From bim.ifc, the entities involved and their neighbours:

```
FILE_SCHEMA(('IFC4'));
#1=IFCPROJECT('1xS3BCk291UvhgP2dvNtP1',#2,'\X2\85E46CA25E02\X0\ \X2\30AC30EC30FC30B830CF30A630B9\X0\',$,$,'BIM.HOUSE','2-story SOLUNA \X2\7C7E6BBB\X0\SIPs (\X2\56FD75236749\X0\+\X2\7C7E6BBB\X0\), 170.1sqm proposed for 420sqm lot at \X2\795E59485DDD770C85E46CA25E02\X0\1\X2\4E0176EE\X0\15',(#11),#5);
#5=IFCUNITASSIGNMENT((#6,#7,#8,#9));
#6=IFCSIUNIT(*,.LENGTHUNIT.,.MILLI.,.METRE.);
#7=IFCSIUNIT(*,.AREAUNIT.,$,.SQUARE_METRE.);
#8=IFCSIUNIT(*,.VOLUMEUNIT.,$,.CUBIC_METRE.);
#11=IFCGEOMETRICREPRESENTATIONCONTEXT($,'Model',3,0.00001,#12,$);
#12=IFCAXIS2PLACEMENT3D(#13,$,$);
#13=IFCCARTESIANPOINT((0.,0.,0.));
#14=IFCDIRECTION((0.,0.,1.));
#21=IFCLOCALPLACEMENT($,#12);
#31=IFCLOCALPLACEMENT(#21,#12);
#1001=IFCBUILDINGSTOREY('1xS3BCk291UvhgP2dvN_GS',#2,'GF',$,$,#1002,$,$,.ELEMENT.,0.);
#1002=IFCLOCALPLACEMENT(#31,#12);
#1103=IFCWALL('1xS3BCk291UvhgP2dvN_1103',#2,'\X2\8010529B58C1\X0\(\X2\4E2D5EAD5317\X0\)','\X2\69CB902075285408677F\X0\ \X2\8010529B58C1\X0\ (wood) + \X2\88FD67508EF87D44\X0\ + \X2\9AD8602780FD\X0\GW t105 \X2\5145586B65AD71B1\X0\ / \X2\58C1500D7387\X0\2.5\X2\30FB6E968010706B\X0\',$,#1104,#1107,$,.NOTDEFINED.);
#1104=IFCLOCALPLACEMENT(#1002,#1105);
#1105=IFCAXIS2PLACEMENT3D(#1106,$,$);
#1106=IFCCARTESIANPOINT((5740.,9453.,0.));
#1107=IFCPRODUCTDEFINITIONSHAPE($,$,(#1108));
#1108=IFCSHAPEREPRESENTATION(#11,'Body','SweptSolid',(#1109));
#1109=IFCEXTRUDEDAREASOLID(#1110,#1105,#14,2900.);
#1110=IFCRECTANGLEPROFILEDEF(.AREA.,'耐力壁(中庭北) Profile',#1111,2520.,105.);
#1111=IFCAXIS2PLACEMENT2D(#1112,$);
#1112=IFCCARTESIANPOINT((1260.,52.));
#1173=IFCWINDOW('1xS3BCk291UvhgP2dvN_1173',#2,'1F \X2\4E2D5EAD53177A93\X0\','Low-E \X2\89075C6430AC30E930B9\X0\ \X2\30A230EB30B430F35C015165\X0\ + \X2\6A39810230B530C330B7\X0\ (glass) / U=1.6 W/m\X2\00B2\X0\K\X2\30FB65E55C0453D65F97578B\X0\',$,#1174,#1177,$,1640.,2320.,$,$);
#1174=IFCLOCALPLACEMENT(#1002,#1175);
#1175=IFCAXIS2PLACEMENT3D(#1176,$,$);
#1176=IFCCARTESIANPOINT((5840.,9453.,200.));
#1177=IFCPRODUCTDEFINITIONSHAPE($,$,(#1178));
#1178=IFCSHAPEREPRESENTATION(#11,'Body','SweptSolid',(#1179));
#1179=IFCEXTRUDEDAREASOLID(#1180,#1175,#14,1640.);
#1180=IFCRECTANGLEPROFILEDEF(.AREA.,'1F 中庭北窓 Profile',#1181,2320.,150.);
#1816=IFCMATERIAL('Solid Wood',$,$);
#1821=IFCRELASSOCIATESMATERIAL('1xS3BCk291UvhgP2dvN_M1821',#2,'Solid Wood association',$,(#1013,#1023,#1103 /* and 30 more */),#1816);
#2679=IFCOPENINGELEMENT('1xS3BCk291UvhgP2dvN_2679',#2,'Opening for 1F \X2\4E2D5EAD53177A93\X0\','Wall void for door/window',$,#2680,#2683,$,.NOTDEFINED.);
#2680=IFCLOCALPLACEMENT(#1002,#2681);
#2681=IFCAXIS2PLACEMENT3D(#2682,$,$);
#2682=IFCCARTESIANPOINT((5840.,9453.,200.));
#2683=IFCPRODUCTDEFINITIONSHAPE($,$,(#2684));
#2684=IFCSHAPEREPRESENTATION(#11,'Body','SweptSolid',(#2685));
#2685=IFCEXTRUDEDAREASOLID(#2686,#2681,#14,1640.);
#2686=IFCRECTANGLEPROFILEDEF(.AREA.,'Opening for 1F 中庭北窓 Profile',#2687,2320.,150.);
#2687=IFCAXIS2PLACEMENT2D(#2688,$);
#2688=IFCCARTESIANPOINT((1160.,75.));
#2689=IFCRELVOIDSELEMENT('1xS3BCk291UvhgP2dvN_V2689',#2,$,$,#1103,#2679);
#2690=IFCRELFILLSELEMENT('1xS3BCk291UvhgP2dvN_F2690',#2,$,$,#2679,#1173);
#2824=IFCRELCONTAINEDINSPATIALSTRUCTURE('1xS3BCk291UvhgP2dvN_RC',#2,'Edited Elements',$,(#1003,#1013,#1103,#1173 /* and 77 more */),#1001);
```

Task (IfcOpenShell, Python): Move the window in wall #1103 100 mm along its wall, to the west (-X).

```python
import ifcopenshell
import ifcopenshell.api.geometry
import ifcopenshell.util.placement
import ifcopenshell.util.unit

model = ifcopenshell.open("bim.ifc")
unit_scale = ifcopenshell.util.unit.calculate_unit_scale(model)

window = model.by_guid("1xS3BCk291UvhgP2dvN_1173")
opening = window.FillsVoids[0].RelatingOpeningElement
wall = opening.VoidsElements[0].RelatingBuildingElement

wall_matrix = ifcopenshell.util.placement.get_local_placement(wall.ObjectPlacement)
shift = wall_matrix[:3, 0] * -0.1 / unit_scale
before = ifcopenshell.util.placement.get_local_placement(window.ObjectPlacement)[:3, 3].copy()

# The window is not placed relative to its opening, so move both.
for product in (opening, window):
    matrix = ifcopenshell.util.placement.get_local_placement(product.ObjectPlacement)
    matrix[:3, 3] += shift
    ifcopenshell.api.geometry.edit_object_placement(model, product=product, matrix=matrix, is_si=False)

after = ifcopenshell.util.placement.get_local_placement(window.ObjectPlacement)[:3, 3]
print("window moved by", (after - before).round(3) + 0.0)

model.write("bim_updated.ifc")
```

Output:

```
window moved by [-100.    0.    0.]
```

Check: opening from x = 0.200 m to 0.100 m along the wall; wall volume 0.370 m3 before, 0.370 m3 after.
